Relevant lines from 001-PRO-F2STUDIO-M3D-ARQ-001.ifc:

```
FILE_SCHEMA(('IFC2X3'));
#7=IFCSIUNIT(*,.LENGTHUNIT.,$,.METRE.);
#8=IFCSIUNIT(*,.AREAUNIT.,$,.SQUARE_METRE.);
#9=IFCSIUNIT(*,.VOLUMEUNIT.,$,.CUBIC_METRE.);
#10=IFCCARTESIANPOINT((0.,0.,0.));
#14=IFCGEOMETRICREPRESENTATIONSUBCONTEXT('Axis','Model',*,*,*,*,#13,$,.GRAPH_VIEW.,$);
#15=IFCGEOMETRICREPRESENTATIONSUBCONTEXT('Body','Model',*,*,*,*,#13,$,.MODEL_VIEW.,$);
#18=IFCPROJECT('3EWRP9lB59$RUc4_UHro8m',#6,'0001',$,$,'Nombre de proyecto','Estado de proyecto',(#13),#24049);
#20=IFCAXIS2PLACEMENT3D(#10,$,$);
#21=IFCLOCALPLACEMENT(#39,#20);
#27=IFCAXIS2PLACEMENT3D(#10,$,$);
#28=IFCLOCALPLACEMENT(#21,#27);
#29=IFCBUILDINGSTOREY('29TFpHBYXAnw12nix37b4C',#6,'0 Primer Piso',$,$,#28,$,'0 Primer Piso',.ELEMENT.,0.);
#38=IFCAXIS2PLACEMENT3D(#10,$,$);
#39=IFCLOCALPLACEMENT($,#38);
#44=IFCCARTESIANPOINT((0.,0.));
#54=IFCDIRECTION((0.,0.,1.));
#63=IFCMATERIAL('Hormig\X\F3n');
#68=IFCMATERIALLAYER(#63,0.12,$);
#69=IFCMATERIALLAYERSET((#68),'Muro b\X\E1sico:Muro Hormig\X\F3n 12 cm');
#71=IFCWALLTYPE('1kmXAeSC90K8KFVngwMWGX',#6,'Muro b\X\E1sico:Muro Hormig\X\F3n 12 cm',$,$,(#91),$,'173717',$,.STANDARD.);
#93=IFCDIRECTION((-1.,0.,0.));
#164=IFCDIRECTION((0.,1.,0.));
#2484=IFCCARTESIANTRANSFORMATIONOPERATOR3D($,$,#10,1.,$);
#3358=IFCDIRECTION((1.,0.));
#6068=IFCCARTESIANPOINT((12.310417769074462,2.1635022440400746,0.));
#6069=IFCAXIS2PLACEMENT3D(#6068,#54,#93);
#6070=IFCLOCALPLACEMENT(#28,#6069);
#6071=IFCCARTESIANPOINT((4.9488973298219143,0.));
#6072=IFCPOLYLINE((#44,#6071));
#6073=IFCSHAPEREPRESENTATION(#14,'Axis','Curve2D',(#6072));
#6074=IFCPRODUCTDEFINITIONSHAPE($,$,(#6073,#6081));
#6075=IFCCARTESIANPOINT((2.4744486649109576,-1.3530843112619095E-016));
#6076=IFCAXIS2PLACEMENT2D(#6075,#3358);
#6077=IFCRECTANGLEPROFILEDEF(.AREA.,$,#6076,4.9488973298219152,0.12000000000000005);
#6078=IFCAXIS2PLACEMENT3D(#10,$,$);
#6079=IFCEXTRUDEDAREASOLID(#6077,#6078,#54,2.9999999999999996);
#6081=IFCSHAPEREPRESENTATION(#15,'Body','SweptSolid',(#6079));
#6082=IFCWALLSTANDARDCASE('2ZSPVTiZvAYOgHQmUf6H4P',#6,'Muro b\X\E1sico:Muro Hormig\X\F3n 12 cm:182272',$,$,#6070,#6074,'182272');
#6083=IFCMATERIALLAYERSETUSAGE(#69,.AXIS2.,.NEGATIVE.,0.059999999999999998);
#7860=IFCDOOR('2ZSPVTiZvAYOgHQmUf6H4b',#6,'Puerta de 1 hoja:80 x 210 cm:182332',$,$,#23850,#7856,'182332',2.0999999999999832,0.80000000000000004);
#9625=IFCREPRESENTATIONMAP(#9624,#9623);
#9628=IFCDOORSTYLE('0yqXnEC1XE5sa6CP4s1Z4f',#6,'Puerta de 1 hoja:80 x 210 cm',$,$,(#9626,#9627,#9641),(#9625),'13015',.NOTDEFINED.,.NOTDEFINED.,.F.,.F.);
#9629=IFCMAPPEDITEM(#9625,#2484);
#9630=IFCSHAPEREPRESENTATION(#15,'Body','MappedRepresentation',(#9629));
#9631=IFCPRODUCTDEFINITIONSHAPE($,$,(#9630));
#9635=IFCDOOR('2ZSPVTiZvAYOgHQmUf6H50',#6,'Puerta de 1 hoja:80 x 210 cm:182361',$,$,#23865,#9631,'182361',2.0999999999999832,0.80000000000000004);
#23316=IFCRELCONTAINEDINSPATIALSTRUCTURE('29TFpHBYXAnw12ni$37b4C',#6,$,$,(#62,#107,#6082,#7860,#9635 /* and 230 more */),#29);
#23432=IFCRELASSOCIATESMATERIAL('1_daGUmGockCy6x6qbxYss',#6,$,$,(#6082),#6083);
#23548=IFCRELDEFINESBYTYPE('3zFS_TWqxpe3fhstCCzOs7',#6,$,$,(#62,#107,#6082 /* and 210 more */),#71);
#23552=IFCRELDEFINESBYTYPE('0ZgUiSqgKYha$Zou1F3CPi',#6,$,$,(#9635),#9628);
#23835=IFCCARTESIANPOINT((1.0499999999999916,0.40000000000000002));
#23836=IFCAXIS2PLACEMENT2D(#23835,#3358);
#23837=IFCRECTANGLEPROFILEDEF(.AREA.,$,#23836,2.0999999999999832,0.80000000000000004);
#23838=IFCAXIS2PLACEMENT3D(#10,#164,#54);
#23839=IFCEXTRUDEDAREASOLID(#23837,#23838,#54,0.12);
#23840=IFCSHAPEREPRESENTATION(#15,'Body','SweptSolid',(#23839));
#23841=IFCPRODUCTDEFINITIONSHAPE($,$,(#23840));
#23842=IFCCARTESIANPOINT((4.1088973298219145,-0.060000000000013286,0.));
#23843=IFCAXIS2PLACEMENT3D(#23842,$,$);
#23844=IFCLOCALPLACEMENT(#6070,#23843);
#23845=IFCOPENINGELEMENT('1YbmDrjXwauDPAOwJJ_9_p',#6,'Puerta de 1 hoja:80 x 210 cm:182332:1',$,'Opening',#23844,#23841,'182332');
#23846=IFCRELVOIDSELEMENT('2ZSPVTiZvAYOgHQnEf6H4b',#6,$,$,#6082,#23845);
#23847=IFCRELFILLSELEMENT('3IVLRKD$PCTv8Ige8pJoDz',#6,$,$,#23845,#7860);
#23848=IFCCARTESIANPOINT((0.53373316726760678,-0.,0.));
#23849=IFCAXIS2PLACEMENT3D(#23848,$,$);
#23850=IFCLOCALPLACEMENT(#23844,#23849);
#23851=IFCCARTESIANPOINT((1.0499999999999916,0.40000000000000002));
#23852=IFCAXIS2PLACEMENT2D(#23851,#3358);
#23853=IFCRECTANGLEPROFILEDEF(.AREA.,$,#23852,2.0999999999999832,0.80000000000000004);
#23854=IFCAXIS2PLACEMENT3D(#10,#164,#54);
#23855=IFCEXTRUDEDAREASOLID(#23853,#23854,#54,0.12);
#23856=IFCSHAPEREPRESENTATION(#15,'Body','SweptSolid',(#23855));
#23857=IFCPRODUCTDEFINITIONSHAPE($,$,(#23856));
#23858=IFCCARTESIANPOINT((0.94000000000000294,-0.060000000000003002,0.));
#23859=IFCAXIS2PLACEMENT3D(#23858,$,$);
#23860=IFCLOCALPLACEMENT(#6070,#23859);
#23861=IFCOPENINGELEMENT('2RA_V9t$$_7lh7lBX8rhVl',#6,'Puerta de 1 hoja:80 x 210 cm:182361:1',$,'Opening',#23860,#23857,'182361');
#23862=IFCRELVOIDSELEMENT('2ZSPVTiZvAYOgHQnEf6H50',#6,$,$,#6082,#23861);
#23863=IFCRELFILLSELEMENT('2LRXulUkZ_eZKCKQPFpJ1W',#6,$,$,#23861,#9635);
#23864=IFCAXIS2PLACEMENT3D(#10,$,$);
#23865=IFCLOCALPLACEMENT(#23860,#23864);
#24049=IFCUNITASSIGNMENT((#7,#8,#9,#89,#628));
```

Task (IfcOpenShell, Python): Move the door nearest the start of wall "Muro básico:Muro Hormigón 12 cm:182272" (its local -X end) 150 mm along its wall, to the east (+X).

```python
import ifcopenshell
import ifcopenshell.api.geometry
import ifcopenshell.util.placement
import ifcopenshell.util.unit

model = ifcopenshell.open("001-PRO-F2STUDIO-M3D-ARQ-001.ifc")
unit_scale = ifcopenshell.util.unit.calculate_unit_scale(model)

door = model.by_guid("2ZSPVTiZvAYOgHQmUf6H50")
opening = door.FillsVoids[0].RelatingOpeningElement
wall = opening.VoidsElements[0].RelatingBuildingElement

wall_matrix = ifcopenshell.util.placement.get_local_placement(wall.ObjectPlacement)
shift = wall_matrix[:3, 0] * -0.15 / unit_scale
before = ifcopenshell.util.placement.get_local_placement(door.ObjectPlacement)[:3, 3].copy()

# The door is placed relative to its opening, so it follows when the opening moves.
matrix = ifcopenshell.util.placement.get_local_placement(opening.ObjectPlacement)
matrix[:3, 3] += shift
ifcopenshell.api.geometry.edit_object_placement(
    model, product=opening, matrix=matrix, is_si=False, should_transform_children=True
)

after = ifcopenshell.util.placement.get_local_placement(door.ObjectPlacement)[:3, 3]
print("door moved by", (after - before).round(3) + 0.0)

model.write("001-PRO-F2STUDIO-M3D-ARQ-001-out.ifc")
```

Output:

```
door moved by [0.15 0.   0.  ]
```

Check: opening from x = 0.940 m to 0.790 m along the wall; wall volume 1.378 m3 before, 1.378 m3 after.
